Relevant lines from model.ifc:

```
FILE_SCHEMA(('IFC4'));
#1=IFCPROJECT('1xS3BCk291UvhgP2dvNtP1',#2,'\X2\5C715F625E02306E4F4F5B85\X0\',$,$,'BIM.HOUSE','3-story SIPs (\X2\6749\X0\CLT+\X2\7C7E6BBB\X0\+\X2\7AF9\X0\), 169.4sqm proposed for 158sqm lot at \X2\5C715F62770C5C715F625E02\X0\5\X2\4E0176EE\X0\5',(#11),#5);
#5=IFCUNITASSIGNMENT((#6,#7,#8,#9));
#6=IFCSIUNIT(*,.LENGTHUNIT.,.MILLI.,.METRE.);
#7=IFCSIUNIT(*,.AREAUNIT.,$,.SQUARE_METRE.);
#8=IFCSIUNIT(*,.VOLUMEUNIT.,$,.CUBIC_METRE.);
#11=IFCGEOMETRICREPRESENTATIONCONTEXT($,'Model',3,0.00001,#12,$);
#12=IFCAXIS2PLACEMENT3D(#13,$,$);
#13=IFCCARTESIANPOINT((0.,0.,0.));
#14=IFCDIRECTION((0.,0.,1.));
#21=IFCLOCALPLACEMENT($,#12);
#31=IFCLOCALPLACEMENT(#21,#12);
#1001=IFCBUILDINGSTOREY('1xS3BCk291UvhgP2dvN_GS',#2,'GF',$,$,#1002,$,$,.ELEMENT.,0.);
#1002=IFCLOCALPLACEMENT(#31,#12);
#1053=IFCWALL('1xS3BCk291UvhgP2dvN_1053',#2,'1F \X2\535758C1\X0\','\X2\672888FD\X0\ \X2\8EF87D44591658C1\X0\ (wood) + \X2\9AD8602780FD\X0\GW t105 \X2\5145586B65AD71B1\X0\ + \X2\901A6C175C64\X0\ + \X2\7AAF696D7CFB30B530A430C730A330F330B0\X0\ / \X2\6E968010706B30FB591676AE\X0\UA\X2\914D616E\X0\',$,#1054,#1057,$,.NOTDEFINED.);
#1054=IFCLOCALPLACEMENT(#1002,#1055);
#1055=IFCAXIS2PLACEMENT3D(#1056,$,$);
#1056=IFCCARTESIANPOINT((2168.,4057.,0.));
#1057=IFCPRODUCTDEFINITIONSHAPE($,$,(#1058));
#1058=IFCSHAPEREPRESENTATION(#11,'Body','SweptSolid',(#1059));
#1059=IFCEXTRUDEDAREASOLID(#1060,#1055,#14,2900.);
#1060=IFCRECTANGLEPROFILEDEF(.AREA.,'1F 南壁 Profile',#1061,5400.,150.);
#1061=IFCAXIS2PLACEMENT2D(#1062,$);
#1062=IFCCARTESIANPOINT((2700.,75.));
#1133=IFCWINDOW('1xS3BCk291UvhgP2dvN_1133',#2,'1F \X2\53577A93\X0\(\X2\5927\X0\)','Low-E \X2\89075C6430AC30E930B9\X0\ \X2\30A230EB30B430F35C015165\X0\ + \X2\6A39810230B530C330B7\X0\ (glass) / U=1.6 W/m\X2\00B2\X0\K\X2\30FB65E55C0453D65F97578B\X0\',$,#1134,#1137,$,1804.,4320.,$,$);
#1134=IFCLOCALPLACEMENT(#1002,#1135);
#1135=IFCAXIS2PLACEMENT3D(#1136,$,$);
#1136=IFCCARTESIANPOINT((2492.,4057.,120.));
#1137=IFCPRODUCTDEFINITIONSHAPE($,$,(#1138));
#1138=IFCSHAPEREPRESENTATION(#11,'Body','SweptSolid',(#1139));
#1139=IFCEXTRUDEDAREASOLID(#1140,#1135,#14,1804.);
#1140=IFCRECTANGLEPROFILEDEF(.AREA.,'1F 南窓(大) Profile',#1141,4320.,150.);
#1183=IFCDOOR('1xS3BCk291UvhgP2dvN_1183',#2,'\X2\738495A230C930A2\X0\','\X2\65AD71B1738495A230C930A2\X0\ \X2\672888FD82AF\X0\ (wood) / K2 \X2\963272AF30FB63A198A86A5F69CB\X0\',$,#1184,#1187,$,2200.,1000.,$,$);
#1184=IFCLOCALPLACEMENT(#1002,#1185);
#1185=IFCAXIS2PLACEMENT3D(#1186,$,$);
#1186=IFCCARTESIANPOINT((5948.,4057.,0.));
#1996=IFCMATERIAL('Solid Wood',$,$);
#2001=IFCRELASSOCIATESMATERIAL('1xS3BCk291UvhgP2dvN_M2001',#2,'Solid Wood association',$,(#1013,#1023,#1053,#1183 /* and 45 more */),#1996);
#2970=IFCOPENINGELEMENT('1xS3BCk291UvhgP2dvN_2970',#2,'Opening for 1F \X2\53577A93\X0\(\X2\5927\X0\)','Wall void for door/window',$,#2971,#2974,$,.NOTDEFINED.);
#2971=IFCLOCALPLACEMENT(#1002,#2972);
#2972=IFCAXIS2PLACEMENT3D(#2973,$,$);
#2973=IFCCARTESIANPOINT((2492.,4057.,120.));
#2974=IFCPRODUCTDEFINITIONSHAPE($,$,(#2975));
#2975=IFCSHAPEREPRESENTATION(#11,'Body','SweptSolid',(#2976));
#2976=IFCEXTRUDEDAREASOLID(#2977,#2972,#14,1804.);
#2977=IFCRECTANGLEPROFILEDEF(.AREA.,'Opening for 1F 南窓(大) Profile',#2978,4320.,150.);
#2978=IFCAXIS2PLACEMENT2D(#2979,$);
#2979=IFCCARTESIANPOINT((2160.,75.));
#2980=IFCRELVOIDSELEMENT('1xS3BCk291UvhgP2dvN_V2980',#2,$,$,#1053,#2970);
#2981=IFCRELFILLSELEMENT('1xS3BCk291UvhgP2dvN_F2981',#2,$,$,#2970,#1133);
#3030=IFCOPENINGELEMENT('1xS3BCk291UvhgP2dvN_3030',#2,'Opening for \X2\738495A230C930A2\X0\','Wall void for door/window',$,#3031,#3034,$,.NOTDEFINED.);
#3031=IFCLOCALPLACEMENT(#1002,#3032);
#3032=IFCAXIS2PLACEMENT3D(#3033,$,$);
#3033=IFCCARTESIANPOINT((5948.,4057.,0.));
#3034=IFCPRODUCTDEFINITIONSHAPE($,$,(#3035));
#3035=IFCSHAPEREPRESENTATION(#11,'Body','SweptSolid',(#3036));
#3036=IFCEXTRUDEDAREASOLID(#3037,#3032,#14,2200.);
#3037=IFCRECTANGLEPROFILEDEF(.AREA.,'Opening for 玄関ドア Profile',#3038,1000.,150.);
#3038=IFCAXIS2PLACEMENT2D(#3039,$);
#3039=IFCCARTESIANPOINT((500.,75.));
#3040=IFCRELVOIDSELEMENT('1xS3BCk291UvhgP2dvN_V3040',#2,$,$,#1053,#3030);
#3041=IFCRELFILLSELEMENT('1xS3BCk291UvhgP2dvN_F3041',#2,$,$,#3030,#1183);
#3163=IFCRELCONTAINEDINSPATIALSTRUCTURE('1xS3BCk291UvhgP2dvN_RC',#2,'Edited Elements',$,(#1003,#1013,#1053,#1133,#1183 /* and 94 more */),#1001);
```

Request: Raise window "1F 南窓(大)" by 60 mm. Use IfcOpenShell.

```python
import numpy as np
import ifcopenshell
import ifcopenshell.api.geometry
import ifcopenshell.util.placement
import ifcopenshell.util.unit

model = ifcopenshell.open("model.ifc")
unit_scale = ifcopenshell.util.unit.calculate_unit_scale(model)

window = model.by_guid("1xS3BCk291UvhgP2dvN_1133")
opening = window.FillsVoids[0].RelatingOpeningElement
dz = 0.06 / unit_scale

shift = np.array([0.0, 0.0, dz])
# The window is not placed relative to its opening, so move both.
for product in (opening, window):
    matrix = ifcopenshell.util.placement.get_local_placement(product.ObjectPlacement)
    matrix[:3, 3] += shift
    ifcopenshell.api.geometry.edit_object_placement(model, product=product, matrix=matrix, is_si=False)

print(f"moved by {dz * unit_scale:+.3f} m")

model.write("model_rev.ifc")
```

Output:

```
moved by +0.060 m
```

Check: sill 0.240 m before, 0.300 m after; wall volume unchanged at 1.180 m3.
